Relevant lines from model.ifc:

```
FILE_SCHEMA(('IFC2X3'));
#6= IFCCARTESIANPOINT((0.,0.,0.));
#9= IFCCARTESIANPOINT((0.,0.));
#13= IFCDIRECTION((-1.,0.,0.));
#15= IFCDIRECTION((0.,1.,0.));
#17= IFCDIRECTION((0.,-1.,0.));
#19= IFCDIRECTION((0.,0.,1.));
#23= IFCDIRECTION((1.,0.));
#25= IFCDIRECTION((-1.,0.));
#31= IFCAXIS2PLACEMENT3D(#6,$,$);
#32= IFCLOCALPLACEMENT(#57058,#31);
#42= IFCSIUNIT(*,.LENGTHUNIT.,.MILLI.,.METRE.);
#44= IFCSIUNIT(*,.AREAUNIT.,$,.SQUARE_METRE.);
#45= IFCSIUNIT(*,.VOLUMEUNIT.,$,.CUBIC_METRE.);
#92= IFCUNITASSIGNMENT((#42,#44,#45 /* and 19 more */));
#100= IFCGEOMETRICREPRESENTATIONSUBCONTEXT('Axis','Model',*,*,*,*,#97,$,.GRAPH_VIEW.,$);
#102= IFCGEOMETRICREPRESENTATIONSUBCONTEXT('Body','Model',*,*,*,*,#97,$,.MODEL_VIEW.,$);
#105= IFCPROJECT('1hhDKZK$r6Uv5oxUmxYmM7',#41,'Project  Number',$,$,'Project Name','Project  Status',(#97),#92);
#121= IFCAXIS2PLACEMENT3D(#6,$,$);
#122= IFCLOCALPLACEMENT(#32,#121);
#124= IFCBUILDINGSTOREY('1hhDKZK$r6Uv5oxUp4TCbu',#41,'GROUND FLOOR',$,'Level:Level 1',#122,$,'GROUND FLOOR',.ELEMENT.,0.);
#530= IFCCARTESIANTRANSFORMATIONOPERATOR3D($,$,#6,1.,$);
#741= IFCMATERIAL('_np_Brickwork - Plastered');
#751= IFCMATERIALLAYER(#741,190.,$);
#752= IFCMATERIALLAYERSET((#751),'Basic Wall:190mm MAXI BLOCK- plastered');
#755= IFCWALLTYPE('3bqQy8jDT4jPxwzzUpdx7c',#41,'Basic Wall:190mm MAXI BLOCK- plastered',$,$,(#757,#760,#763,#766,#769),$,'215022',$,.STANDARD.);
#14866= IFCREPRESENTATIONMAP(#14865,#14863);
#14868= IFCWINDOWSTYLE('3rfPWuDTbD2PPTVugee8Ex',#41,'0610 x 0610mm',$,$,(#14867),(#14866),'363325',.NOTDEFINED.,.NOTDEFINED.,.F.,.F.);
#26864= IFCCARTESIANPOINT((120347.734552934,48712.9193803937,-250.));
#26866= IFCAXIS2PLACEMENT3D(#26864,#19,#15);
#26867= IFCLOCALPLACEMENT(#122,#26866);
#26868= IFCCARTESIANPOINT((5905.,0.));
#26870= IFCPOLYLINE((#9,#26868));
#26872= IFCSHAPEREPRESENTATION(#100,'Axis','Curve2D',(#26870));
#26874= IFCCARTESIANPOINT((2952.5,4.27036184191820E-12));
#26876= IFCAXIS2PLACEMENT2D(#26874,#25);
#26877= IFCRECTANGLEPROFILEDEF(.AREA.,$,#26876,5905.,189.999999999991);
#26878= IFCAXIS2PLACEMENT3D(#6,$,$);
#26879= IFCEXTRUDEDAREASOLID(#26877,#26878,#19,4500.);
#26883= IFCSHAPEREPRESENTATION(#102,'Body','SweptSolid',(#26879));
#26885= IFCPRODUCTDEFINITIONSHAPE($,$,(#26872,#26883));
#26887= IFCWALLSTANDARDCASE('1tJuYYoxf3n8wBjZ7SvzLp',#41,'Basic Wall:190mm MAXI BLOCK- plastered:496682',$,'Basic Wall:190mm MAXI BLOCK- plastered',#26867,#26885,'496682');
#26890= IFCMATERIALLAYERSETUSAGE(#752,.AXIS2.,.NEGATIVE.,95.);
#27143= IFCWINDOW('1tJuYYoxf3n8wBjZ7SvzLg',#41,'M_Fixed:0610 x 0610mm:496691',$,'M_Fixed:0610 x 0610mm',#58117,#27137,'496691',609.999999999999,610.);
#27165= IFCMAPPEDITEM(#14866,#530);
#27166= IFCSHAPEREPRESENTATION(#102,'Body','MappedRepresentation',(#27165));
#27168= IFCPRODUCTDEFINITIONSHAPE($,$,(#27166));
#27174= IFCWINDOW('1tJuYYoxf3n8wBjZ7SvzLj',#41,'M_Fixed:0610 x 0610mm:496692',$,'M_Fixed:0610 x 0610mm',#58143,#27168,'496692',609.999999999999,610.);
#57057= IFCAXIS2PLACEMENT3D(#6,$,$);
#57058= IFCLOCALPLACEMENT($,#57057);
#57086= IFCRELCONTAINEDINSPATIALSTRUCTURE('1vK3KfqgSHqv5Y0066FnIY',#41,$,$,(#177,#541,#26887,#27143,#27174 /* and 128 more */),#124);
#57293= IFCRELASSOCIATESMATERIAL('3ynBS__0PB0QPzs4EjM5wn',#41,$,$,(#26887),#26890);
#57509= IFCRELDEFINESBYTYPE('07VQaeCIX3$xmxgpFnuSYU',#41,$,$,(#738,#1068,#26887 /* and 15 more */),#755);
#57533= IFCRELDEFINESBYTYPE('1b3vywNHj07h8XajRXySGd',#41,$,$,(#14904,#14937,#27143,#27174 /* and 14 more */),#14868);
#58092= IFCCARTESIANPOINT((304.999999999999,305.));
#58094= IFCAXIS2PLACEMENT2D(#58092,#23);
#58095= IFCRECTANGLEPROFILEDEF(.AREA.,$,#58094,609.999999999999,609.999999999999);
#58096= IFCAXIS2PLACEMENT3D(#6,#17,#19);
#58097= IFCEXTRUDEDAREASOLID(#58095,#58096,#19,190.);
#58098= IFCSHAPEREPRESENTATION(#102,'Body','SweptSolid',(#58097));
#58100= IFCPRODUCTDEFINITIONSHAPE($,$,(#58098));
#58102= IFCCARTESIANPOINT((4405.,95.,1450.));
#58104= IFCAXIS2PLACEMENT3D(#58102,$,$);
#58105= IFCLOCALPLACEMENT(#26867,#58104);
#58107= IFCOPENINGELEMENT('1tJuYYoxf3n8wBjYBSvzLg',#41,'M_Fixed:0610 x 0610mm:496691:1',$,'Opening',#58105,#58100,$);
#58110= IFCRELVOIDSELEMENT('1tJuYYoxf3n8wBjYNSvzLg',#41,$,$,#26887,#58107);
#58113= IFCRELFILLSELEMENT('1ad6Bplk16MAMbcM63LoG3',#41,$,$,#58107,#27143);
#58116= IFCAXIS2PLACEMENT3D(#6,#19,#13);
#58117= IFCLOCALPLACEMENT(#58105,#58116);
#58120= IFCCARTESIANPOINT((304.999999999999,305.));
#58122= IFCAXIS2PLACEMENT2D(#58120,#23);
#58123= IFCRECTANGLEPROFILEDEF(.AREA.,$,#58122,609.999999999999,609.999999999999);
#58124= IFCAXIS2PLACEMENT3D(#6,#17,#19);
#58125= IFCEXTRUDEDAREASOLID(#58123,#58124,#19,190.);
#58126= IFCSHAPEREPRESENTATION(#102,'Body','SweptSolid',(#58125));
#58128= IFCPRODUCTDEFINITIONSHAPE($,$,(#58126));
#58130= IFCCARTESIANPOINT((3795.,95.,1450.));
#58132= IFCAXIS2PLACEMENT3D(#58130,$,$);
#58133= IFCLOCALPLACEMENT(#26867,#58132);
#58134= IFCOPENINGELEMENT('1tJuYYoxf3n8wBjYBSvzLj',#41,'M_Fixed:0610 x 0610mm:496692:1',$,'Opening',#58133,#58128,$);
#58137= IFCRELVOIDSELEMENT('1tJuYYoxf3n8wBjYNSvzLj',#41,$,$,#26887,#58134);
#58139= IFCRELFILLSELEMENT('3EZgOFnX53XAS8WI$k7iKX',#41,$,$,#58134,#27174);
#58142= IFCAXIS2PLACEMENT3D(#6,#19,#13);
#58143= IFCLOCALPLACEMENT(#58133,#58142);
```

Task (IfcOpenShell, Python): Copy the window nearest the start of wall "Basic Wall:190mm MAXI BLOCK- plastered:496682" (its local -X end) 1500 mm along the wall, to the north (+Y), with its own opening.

```python
import ifcopenshell
import ifcopenshell.api.feature
import ifcopenshell.api.geometry
import ifcopenshell.api.root
import ifcopenshell.geom
import ifcopenshell.util.element
import ifcopenshell.util.placement
import ifcopenshell.util.shape
import ifcopenshell.util.unit

model = ifcopenshell.open("model.ifc")
unit_scale = ifcopenshell.util.unit.calculate_unit_scale(model)
settings = ifcopenshell.geom.settings()


def volume(element):
    """Net volume in cubic metres, openings subtracted."""
    shape = ifcopenshell.geom.create_shape(settings, element)
    return ifcopenshell.util.shape.get_volume(shape.geometry)


def reuse_history(source, copy):
    """copy_class also copies each property set's owner history, people and application; keep the originals."""
    for rel in copy.IsDefinedBy:
        if rel.is_a("IfcRelDefinesByProperties") and (history := rel.RelatingPropertyDefinition.OwnerHistory):
            rel.RelatingPropertyDefinition.OwnerHistory = source.OwnerHistory
            ifcopenshell.util.element.remove_deep2(model, history)


window = model.by_id(27174)
opening = window.FillsVoids[0].RelatingOpeningElement
wall = opening.VoidsElements[0].RelatingBuildingElement
before = volume(wall)
shift = ifcopenshell.util.placement.get_local_placement(wall.ObjectPlacement)[:3, 0] * 1.5 / unit_scale

# copy_class copies the void relationship, type, container and properties, but no geometry.
new_opening = ifcopenshell.api.root.copy_class(model, product=opening)
new_opening.Representation = ifcopenshell.util.element.copy_deep(
    model, opening.Representation, exclude=["IfcGeometricRepresentationContext", "IfcRepresentationMap"]
)
new_opening.Name = "M_Fixed:0610 x 0610mm"
new_window = ifcopenshell.api.root.copy_class(model, product=window)
new_window.Representation = ifcopenshell.util.element.copy_deep(
    model, window.Representation, exclude=["IfcGeometricRepresentationContext", "IfcRepresentationMap"]
)
new_window.Name = "M_Fixed:0610 x 0610mm"
new_window.Tag = None
reuse_history(window, new_window)
fills = ifcopenshell.api.feature.add_filling(model, opening=new_opening, element=new_window)
fills.OwnerHistory = new_window.OwnerHistory  # required in IFC2X3

for old, new in ((opening, new_opening), (window, new_window)):
    matrix = ifcopenshell.util.placement.get_local_placement(old.ObjectPlacement)
    matrix[:3, 3] += shift
    ifcopenshell.api.geometry.edit_object_placement(model, product=new, matrix=matrix, is_si=False)

after = volume(wall)

print(f"wall volume {before:.3f} -> {after:.3f} m3")

model.write("model_v2.ifc")
```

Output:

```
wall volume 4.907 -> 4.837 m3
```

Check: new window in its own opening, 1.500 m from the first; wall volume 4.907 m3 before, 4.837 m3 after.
